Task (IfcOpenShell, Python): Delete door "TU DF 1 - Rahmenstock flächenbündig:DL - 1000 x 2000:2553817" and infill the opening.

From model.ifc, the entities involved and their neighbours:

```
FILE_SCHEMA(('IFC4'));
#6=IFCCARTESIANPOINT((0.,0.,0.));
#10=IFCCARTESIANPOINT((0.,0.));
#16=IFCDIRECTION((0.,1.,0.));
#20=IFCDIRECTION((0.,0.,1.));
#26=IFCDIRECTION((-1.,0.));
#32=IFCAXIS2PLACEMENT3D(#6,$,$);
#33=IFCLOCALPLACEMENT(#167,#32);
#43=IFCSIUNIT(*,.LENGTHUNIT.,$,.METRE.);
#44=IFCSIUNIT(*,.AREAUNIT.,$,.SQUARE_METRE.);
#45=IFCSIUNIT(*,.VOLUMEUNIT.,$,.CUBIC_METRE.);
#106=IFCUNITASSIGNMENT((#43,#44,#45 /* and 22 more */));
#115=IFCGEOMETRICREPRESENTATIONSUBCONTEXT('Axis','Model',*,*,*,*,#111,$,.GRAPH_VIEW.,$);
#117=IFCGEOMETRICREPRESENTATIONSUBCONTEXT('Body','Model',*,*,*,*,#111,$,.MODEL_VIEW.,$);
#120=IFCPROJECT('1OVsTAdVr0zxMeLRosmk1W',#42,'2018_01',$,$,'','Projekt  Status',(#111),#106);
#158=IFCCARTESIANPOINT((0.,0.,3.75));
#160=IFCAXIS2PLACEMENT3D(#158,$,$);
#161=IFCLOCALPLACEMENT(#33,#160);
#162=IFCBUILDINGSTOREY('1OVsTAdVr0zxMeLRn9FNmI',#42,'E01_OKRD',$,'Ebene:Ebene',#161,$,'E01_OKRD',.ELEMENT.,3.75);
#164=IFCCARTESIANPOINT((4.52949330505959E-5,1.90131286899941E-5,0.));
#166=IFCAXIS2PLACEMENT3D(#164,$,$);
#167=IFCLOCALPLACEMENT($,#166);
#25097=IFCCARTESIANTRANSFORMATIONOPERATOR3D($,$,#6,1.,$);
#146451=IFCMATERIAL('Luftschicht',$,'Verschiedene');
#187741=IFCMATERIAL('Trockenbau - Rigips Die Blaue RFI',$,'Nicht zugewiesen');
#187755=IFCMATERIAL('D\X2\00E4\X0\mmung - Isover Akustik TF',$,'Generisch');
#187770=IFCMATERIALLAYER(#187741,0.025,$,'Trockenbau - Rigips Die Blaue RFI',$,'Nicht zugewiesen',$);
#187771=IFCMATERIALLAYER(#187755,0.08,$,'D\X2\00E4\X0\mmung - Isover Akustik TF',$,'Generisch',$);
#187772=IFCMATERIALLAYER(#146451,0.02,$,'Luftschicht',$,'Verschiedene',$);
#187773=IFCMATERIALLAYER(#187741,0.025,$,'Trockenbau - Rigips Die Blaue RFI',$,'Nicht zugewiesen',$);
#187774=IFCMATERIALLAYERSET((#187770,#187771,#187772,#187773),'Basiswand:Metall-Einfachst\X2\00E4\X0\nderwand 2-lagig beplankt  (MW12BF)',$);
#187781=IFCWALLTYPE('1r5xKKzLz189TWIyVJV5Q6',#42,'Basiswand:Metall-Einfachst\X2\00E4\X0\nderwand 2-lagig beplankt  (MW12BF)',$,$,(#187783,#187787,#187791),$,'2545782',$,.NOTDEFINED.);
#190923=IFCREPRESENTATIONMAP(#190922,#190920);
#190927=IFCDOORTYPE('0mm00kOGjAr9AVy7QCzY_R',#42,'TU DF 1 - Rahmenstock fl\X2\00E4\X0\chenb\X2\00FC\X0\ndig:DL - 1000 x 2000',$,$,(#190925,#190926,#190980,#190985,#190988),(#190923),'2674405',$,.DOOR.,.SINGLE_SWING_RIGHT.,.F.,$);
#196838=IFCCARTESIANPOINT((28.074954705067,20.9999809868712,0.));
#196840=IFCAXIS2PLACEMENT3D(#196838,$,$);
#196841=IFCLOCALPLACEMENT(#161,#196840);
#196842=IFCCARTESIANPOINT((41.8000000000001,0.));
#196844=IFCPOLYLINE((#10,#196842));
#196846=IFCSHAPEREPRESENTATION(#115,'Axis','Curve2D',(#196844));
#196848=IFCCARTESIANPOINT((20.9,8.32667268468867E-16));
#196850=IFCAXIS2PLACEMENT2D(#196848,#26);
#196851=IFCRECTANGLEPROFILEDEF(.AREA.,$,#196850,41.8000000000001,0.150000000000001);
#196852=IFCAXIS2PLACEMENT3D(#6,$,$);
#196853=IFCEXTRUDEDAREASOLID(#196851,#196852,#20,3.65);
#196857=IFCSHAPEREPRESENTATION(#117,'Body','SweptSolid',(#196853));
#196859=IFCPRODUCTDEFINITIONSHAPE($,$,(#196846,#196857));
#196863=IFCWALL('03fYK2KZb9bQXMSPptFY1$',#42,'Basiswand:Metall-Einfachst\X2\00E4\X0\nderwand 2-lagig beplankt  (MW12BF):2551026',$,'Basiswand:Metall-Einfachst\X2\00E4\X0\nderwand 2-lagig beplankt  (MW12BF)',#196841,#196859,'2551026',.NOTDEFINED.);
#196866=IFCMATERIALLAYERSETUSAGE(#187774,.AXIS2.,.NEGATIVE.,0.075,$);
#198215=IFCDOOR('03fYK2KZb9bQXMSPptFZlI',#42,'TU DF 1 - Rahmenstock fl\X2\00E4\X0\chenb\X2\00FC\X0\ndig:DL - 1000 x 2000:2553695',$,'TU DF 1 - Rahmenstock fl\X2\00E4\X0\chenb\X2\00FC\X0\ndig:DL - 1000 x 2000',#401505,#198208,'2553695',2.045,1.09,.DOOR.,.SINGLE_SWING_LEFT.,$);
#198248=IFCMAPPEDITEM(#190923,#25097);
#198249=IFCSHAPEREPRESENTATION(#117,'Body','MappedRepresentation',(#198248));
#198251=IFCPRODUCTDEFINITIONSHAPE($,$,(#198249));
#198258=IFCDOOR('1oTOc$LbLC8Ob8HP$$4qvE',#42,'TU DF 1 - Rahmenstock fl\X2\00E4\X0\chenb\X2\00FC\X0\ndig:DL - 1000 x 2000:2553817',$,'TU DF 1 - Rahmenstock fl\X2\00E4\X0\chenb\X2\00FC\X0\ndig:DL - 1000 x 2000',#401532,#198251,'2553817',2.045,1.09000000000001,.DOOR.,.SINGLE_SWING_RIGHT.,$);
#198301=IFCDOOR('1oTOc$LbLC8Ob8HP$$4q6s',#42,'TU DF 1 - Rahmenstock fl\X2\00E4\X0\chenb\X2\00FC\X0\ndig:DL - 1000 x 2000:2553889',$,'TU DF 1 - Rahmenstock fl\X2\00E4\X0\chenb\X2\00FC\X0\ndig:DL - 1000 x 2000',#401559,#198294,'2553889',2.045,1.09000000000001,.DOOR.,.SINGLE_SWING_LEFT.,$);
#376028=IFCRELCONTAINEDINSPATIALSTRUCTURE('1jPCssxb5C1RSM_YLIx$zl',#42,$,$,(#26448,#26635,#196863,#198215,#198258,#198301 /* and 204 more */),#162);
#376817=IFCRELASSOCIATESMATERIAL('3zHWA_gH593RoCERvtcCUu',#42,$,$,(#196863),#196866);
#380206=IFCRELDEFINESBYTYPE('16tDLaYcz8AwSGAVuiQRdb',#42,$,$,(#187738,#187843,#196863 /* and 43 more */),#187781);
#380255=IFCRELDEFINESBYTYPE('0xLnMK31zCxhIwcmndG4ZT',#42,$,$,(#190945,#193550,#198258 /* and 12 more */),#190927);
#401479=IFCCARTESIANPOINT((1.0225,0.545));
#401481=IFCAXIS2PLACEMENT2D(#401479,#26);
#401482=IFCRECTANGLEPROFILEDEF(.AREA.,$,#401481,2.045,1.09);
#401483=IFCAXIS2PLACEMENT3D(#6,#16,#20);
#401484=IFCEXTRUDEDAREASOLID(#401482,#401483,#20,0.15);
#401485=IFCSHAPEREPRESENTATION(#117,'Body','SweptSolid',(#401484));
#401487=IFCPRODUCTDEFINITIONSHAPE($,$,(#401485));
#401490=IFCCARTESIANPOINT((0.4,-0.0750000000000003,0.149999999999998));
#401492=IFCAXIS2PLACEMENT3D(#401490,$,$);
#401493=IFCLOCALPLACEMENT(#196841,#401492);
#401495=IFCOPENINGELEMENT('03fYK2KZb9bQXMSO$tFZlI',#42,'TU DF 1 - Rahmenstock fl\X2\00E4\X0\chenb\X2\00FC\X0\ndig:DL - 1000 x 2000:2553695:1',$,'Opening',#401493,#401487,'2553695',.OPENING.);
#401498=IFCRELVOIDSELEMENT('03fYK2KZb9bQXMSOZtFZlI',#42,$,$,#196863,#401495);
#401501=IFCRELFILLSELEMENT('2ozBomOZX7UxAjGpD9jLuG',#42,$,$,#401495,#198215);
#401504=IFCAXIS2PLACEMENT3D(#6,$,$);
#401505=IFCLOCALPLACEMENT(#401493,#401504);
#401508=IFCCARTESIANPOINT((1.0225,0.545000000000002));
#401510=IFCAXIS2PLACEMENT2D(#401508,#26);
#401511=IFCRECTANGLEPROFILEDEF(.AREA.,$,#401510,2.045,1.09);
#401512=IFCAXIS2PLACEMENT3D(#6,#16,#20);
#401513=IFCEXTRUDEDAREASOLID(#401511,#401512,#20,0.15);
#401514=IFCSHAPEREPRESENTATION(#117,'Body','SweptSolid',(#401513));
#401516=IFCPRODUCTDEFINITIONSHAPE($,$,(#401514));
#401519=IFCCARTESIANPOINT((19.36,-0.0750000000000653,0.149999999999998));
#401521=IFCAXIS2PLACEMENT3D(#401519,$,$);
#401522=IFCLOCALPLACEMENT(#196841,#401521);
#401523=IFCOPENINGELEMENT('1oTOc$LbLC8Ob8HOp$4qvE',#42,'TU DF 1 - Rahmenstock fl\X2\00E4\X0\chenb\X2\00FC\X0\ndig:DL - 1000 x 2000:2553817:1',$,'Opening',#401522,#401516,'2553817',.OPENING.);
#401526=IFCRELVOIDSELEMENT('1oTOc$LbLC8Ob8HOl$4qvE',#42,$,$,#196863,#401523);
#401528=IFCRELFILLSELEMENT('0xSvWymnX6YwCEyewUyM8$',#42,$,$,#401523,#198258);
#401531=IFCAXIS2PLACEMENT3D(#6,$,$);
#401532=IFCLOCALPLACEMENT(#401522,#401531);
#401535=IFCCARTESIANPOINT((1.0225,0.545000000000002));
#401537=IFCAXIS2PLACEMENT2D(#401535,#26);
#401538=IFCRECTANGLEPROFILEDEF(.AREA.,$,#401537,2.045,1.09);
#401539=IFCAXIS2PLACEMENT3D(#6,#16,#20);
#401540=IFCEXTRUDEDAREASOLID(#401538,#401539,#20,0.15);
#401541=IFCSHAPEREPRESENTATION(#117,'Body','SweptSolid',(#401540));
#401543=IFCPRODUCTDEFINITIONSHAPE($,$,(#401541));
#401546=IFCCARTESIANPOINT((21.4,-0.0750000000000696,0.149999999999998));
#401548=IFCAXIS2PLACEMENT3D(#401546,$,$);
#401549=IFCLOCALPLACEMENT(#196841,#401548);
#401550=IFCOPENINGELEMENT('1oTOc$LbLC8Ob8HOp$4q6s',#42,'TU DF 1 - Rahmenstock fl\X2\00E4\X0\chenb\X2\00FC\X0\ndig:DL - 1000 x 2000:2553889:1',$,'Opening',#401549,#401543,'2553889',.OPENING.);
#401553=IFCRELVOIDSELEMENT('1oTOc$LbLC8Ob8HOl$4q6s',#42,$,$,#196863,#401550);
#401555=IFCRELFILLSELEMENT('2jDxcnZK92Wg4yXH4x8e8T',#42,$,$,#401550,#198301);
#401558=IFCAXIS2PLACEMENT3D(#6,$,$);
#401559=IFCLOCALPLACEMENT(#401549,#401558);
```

```python
import ifcopenshell
import ifcopenshell.api.feature
import ifcopenshell.api.root
import ifcopenshell.geom
import ifcopenshell.util.shape

model = ifcopenshell.open("model.ifc")
settings = ifcopenshell.geom.settings()


def volume(element):
    """Net volume in cubic metres, openings subtracted."""
    shape = ifcopenshell.geom.create_shape(settings, element)
    return ifcopenshell.util.shape.get_volume(shape.geometry)


door = model.by_guid("1oTOc$LbLC8Ob8HP$$4qvE")
opening = door.FillsVoids[0].RelatingOpeningElement
wall = opening.VoidsElements[0].RelatingBuildingElement
before = volume(wall)

ifcopenshell.api.root.remove_product(model, product=door)
ifcopenshell.api.feature.remove_feature(model, feature=opening)

after = volume(wall)

print(f"wall volume {before:.3f} -> {after:.3f} m3")

model.write("model_updated.ifc")
```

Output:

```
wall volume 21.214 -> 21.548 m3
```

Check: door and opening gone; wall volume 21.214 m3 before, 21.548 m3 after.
